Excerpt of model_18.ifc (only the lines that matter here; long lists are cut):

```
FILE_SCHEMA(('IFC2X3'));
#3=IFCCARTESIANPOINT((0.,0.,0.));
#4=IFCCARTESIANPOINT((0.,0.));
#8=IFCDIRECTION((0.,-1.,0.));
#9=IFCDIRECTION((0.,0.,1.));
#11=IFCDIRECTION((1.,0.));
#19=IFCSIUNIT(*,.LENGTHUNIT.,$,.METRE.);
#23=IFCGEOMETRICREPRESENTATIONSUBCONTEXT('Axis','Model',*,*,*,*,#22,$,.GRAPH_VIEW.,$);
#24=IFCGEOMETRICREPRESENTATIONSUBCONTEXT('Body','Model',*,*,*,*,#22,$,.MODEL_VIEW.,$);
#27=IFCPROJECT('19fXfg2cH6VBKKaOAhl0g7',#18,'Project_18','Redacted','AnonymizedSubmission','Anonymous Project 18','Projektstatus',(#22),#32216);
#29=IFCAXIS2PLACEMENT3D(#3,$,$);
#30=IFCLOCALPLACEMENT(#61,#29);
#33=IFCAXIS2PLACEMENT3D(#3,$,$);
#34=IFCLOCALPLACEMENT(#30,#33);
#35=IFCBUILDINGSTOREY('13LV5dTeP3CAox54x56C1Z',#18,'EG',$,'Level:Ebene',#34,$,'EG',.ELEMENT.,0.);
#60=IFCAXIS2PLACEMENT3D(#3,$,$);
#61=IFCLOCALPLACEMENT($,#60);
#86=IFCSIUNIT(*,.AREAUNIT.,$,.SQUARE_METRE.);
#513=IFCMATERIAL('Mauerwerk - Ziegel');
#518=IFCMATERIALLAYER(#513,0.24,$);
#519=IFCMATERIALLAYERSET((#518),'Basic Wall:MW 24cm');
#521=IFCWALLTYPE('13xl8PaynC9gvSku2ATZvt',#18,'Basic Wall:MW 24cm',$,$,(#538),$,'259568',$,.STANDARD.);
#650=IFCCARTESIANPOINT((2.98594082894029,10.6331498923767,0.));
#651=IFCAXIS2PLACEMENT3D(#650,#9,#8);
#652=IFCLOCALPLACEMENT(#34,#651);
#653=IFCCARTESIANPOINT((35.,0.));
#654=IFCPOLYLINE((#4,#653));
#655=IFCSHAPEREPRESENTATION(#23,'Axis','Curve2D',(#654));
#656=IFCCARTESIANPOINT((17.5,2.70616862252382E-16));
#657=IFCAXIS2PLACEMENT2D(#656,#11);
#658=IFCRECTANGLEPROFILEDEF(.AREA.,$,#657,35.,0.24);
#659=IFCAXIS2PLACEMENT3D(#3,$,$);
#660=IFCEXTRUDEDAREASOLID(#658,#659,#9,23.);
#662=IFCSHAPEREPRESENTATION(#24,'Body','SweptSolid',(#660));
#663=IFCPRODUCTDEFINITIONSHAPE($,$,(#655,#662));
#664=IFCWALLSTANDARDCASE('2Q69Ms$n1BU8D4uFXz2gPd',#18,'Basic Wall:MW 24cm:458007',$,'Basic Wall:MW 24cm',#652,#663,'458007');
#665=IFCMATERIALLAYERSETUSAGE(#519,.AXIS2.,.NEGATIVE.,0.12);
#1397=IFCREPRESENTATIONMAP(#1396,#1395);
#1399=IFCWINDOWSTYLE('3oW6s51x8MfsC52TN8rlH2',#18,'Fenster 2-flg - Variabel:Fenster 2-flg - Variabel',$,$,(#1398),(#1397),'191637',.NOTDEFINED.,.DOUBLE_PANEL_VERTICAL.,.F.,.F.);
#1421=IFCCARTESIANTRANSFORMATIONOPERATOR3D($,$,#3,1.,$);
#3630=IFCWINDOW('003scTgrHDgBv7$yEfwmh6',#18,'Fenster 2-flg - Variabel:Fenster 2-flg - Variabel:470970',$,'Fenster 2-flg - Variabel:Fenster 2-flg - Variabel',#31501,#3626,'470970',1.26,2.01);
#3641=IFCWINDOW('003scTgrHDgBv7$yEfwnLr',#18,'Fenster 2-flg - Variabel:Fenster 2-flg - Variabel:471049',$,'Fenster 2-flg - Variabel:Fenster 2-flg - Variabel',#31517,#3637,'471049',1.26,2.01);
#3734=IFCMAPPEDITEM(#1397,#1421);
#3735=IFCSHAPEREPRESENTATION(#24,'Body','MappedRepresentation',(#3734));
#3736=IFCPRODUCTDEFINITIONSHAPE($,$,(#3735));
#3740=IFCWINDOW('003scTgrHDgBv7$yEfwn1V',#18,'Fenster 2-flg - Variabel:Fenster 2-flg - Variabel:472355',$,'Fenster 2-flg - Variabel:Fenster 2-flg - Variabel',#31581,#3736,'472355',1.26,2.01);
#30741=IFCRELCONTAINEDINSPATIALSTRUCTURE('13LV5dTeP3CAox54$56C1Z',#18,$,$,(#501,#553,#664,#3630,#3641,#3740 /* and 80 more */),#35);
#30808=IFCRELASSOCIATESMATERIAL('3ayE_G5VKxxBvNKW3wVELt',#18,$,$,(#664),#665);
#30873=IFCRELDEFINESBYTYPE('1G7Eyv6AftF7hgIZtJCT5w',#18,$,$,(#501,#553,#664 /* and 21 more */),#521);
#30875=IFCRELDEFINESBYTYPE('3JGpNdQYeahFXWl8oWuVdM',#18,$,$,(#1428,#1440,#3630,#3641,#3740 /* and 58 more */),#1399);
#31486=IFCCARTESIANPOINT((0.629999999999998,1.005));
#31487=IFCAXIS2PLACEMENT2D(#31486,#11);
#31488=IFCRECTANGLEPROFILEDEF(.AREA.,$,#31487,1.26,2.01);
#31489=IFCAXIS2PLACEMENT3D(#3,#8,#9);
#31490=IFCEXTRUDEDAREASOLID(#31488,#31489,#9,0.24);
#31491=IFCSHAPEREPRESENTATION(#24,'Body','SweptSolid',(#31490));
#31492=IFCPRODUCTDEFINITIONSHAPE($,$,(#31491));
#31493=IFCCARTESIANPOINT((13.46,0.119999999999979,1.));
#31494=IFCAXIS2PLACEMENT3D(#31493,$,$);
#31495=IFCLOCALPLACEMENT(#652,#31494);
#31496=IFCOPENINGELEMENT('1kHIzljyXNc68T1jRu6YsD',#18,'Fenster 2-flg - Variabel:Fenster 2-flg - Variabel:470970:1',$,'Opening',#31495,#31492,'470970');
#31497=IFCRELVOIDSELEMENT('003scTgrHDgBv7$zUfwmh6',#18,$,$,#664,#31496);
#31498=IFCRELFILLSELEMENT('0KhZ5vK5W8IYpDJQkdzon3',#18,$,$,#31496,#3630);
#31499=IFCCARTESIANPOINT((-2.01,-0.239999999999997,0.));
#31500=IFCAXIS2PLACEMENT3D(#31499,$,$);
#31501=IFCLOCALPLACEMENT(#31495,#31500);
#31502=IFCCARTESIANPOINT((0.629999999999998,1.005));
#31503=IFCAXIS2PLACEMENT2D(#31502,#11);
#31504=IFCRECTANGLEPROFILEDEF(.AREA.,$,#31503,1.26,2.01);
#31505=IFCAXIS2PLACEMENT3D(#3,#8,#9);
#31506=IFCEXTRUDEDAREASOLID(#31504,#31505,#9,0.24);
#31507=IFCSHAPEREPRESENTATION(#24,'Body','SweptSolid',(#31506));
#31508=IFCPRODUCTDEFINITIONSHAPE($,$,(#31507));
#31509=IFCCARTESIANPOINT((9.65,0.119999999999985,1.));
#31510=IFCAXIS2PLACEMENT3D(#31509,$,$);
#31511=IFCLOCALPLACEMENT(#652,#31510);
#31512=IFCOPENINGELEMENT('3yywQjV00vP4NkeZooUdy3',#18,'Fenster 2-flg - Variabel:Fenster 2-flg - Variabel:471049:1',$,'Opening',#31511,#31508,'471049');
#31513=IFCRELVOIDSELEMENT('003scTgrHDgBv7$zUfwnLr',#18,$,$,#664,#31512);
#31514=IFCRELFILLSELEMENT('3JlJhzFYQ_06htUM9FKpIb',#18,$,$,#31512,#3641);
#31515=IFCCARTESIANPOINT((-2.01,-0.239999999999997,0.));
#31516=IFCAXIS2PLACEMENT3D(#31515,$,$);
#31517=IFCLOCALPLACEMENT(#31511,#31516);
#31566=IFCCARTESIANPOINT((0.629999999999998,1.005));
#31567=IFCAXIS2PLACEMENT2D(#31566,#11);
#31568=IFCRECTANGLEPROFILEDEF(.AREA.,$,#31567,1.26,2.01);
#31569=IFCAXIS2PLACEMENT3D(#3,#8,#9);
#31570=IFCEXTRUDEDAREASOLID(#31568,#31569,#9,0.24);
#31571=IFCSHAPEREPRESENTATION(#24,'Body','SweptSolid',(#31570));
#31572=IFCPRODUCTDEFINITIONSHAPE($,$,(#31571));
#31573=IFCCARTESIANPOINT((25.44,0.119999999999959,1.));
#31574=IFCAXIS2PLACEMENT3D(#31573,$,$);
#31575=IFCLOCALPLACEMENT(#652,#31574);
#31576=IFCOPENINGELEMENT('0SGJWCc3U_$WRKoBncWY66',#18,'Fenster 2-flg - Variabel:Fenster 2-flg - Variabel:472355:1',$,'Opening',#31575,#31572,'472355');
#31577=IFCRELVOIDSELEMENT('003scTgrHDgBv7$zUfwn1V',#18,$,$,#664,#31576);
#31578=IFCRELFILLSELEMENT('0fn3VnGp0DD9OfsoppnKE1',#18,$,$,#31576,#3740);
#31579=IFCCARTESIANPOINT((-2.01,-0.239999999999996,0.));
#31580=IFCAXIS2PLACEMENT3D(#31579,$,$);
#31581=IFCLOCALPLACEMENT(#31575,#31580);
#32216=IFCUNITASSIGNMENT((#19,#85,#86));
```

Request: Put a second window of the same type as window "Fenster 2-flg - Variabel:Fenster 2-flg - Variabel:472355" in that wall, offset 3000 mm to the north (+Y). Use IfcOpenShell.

```python
import ifcopenshell
import ifcopenshell.api.feature
import ifcopenshell.api.geometry
import ifcopenshell.api.root
import ifcopenshell.geom
import ifcopenshell.util.element
import ifcopenshell.util.placement
import ifcopenshell.util.shape

model = ifcopenshell.open("model_18.ifc")
settings = ifcopenshell.geom.settings()


def volume(element):
    """Net volume in cubic metres, openings subtracted."""
    shape = ifcopenshell.geom.create_shape(settings, element)
    return ifcopenshell.util.shape.get_volume(shape.geometry)


def reuse_history(source, copy):
    """copy_class also copies each property set's owner history, people and application; keep the originals."""
    for rel in copy.IsDefinedBy:
        if rel.is_a("IfcRelDefinesByProperties") and (history := rel.RelatingPropertyDefinition.OwnerHistory):
            rel.RelatingPropertyDefinition.OwnerHistory = source.OwnerHistory
            ifcopenshell.util.element.remove_deep2(model, history)


window = model.by_guid("003scTgrHDgBv7$yEfwn1V")
opening = window.FillsVoids[0].RelatingOpeningElement
wall = opening.VoidsElements[0].RelatingBuildingElement
before = volume(wall)
shift = ifcopenshell.util.placement.get_local_placement(wall.ObjectPlacement)[:3, 0] * -3.0

# copy_class copies the void relationship, type, container and properties, but no geometry.
new_opening = ifcopenshell.api.root.copy_class(model, product=opening)
new_opening.Representation = ifcopenshell.util.element.copy_deep(
    model, opening.Representation, exclude=["IfcGeometricRepresentationContext", "IfcRepresentationMap"]
)
new_opening.Name = "Fenster 2-flg - Variabel:Fenster 2-flg - Variabel"
new_opening.Tag = None
new_window = ifcopenshell.api.root.copy_class(model, product=window)
new_window.Representation = ifcopenshell.util.element.copy_deep(
    model, window.Representation, exclude=["IfcGeometricRepresentationContext", "IfcRepresentationMap"]
)
new_window.Name = "Fenster 2-flg - Variabel:Fenster 2-flg - Variabel"
new_window.Tag = None
reuse_history(window, new_window)
fills = ifcopenshell.api.feature.add_filling(model, opening=new_opening, element=new_window)
fills.OwnerHistory = new_window.OwnerHistory  # required in IFC2X3

for old, new in ((opening, new_opening), (window, new_window)):
    matrix = ifcopenshell.util.placement.get_local_placement(old.ObjectPlacement)
    matrix[:3, 3] += shift
    ifcopenshell.api.geometry.edit_object_placement(model, product=new, matrix=matrix, is_si=False)

after = volume(wall)

print(f"wall volume {before:.3f} -> {after:.3f} m3")

model.write("model_18-out.ifc")
```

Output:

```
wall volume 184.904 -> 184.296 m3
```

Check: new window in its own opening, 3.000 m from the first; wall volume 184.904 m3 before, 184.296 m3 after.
